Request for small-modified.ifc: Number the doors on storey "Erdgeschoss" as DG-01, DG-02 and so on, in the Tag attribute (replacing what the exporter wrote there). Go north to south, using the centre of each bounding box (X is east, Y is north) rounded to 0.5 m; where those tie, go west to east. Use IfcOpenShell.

First a look at what the model holds.

```python
import ifcopenshell
import ifcopenshell.util.element
import ifcopenshell.util.placement

model = ifcopenshell.open("small-modified.ifc")
print(model.schema)
storey = next(s for s in model.by_type("IfcBuildingStorey") if s.Name == "Erdgeschoss")
doors = [e for e in ifcopenshell.util.element.get_decomposition(storey) if e.is_a("IfcDoor")]
for e in sorted(doors, key=lambda e: e.id()):
    origin = ifcopenshell.util.placement.get_local_placement(e.ObjectPlacement)[:3, 3]
    print(e.id(), e.Tag, e.Name, origin.round(2) + 0.0, sep=" | ")
```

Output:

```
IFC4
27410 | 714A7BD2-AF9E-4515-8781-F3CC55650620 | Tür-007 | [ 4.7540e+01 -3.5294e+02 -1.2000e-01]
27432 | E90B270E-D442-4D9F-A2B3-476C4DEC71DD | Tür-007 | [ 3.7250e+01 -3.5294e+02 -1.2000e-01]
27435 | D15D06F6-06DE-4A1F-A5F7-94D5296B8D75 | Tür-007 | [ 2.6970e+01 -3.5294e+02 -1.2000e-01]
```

```python
import ifcopenshell
import ifcopenshell.geom
import ifcopenshell.util.element
import ifcopenshell.util.shape

model = ifcopenshell.open("small-modified.ifc")
settings = ifcopenshell.geom.settings()
settings.set("use-world-coords", True)


def centre(element):
    shape = ifcopenshell.geom.create_shape(settings, element)
    return ifcopenshell.util.shape.get_bbox_centroid(shape.geometry)


storey = next(s for s in model.by_type("IfcBuildingStorey") if s.Name == "Erdgeschoss")
doors = [e for e in ifcopenshell.util.element.get_decomposition(storey) if e.is_a("IfcDoor")]

# Insertion points can sit at a corner or the storey origin, so sort by the geometry (in metres).
centres = {e: centre(e) for e in doors}
doors.sort(key=lambda e: (-round(centres[e][1] / 0.5), centres[e][0]))

for i, e in enumerate(doors, start=1):
    number = f"DG-{i:02d}"
    e.Tag = number
    print(e.id(), number)

model.write("small-modified_rev.ifc")
```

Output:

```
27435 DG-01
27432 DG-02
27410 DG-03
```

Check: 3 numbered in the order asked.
